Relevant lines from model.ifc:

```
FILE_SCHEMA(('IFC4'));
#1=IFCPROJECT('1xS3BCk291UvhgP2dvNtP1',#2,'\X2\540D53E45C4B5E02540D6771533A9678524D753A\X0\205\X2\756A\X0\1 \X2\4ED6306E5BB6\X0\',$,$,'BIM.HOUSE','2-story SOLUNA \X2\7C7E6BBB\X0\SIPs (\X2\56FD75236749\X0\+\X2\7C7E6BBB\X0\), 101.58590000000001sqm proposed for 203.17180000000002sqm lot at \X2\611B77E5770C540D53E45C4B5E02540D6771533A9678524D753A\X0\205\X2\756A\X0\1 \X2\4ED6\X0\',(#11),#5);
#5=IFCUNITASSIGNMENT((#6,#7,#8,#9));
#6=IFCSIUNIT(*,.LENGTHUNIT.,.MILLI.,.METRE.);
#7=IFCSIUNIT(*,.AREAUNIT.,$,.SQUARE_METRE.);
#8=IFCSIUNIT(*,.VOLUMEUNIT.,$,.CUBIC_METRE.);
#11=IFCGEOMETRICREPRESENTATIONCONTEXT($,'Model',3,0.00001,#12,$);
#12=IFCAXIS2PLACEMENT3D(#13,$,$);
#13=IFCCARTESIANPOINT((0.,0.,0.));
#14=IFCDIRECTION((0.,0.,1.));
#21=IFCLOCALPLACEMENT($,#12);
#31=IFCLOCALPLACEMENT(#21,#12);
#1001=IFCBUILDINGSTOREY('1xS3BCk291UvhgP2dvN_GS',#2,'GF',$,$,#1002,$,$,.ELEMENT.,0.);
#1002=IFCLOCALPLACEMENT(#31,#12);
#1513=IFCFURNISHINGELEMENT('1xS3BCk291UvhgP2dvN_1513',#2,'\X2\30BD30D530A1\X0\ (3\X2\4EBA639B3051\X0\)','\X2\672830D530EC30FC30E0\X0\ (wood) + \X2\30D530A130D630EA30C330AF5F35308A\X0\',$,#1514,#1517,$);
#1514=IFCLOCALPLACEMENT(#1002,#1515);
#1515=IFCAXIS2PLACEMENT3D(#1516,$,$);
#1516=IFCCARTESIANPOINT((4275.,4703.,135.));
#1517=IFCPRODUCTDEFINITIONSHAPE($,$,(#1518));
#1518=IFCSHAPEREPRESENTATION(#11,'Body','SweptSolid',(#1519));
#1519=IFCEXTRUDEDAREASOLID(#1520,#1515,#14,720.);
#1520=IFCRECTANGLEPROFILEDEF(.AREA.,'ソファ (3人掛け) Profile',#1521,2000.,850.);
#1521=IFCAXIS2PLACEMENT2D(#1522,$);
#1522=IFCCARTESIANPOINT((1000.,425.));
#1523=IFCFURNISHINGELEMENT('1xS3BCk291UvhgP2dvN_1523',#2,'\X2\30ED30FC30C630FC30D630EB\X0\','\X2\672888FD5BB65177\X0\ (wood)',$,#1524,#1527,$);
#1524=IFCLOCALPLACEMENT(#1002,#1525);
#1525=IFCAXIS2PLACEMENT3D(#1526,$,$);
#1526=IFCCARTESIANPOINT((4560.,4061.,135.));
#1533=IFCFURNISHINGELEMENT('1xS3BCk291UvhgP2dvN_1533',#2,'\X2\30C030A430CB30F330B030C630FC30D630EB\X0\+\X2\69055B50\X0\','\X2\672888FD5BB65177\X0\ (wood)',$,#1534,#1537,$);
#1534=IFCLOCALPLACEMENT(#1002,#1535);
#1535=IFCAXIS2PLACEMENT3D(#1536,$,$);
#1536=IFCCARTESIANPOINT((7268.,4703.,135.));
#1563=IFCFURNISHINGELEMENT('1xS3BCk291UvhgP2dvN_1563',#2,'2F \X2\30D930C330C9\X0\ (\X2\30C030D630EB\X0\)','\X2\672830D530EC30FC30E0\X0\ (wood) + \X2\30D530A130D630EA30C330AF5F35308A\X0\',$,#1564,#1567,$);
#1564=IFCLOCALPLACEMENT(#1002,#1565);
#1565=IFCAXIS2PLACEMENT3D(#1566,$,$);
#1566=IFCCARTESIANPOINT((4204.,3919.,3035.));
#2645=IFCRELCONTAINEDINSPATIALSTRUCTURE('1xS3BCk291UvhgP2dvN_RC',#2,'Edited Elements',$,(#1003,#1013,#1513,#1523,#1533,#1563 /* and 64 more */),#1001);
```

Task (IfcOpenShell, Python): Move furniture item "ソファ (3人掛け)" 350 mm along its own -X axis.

```python
import ifcopenshell
import ifcopenshell.api.geometry
import ifcopenshell.util.placement

model = ifcopenshell.open("model.ifc")

item = model.by_guid("1xS3BCk291UvhgP2dvN_1513")
matrix = ifcopenshell.util.placement.get_local_placement(item.ObjectPlacement)
matrix[:3, 3] -= matrix[:3, 0] * 350.0
ifcopenshell.api.geometry.edit_object_placement(model, product=item, matrix=matrix, is_si=False)

print(ifcopenshell.util.placement.get_local_placement(item.ObjectPlacement).round(3) + 0.0)

model.write("model_updated.ifc")
```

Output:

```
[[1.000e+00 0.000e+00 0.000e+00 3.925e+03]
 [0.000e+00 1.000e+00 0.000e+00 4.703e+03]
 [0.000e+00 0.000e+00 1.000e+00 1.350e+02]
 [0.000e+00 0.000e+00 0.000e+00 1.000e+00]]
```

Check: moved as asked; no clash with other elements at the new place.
